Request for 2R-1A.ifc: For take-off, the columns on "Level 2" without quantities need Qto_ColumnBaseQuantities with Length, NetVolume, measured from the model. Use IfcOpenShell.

First a look at what the model holds.

```python
import ifcopenshell
import ifcopenshell.util.element
import ifcopenshell.util.unit

model = ifcopenshell.open("2R-1A.ifc")
print(model.schema)
for unit_type in ("LENGTHUNIT", "AREAUNIT", "VOLUMEUNIT"):
    print(unit_type, ifcopenshell.util.unit.calculate_unit_scale(model, unit_type))
storey = next(s for s in model.by_type("IfcBuildingStorey") if s.Name == "Level 2")
columns = [e for e in ifcopenshell.util.element.get_decomposition(storey) if e.is_a("IfcColumn")]
for e in sorted(columns, key=lambda e: e.id()):
    print(e.id(), e.is_a(), e.Name, list(ifcopenshell.util.element.get_psets(e, qtos_only=True)), sep=" | ")
```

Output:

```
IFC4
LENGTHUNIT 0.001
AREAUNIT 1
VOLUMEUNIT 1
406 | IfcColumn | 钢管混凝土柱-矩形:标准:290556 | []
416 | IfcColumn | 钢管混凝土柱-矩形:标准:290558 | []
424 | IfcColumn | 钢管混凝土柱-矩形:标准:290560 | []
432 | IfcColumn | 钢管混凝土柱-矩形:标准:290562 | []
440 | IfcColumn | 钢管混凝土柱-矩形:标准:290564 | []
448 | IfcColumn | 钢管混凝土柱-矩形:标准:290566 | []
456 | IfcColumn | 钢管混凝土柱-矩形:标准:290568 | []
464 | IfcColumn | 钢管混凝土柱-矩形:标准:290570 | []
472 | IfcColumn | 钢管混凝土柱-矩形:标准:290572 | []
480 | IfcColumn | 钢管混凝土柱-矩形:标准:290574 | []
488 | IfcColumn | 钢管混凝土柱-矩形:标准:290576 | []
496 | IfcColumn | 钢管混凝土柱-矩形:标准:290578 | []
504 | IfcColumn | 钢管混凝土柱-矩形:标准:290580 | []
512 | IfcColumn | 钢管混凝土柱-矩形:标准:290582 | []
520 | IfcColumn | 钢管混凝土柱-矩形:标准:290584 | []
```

```python
import ifcopenshell
import ifcopenshell.api.pset
import ifcopenshell.geom
import ifcopenshell.util.element
import ifcopenshell.util.shape
import ifcopenshell.util.unit

model = ifcopenshell.open("2R-1A.ifc")
unit_scale = ifcopenshell.util.unit.calculate_unit_scale(model)
volume_scale = ifcopenshell.util.unit.calculate_unit_scale(model, "VOLUMEUNIT")
settings = ifcopenshell.geom.settings()

storey = next(s for s in model.by_type("IfcBuildingStorey") if s.Name == "Level 2")
columns = [e for e in ifcopenshell.util.element.get_decomposition(storey) if e.is_a("IfcColumn")]

for e in sorted(columns, key=lambda e: e.id()):
    if ifcopenshell.util.element.get_psets(e, qtos_only=True, should_inherit=False):
        continue
    # Geometry comes back in metres, in the element's own axes.
    shape = ifcopenshell.geom.create_shape(settings, e)
    values = {
        "Length": ifcopenshell.util.shape.get_z(shape.geometry) / unit_scale,
        "NetVolume": ifcopenshell.util.shape.get_volume(shape.geometry) / volume_scale,
    }
    qto = ifcopenshell.api.pset.add_qto(model, product=e, name="Qto_ColumnBaseQuantities")
    ifcopenshell.api.pset.edit_qto(model, qto=qto, properties=values)
    print(e.id(), {k: round(v, 3) for k, v in values.items()})

model.write("2R-1A_edited.ifc")
```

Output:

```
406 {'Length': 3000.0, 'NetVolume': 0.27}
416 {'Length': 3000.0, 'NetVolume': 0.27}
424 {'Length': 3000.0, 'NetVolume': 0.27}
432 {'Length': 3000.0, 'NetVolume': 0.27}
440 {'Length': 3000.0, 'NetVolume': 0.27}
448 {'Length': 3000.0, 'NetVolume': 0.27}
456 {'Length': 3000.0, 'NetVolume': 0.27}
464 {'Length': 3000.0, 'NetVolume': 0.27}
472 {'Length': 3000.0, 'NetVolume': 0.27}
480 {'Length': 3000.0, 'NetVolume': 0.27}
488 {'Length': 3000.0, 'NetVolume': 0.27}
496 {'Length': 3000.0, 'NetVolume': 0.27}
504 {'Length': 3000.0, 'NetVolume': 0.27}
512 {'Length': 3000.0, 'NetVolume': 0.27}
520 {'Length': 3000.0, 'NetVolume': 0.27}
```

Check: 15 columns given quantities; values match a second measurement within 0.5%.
